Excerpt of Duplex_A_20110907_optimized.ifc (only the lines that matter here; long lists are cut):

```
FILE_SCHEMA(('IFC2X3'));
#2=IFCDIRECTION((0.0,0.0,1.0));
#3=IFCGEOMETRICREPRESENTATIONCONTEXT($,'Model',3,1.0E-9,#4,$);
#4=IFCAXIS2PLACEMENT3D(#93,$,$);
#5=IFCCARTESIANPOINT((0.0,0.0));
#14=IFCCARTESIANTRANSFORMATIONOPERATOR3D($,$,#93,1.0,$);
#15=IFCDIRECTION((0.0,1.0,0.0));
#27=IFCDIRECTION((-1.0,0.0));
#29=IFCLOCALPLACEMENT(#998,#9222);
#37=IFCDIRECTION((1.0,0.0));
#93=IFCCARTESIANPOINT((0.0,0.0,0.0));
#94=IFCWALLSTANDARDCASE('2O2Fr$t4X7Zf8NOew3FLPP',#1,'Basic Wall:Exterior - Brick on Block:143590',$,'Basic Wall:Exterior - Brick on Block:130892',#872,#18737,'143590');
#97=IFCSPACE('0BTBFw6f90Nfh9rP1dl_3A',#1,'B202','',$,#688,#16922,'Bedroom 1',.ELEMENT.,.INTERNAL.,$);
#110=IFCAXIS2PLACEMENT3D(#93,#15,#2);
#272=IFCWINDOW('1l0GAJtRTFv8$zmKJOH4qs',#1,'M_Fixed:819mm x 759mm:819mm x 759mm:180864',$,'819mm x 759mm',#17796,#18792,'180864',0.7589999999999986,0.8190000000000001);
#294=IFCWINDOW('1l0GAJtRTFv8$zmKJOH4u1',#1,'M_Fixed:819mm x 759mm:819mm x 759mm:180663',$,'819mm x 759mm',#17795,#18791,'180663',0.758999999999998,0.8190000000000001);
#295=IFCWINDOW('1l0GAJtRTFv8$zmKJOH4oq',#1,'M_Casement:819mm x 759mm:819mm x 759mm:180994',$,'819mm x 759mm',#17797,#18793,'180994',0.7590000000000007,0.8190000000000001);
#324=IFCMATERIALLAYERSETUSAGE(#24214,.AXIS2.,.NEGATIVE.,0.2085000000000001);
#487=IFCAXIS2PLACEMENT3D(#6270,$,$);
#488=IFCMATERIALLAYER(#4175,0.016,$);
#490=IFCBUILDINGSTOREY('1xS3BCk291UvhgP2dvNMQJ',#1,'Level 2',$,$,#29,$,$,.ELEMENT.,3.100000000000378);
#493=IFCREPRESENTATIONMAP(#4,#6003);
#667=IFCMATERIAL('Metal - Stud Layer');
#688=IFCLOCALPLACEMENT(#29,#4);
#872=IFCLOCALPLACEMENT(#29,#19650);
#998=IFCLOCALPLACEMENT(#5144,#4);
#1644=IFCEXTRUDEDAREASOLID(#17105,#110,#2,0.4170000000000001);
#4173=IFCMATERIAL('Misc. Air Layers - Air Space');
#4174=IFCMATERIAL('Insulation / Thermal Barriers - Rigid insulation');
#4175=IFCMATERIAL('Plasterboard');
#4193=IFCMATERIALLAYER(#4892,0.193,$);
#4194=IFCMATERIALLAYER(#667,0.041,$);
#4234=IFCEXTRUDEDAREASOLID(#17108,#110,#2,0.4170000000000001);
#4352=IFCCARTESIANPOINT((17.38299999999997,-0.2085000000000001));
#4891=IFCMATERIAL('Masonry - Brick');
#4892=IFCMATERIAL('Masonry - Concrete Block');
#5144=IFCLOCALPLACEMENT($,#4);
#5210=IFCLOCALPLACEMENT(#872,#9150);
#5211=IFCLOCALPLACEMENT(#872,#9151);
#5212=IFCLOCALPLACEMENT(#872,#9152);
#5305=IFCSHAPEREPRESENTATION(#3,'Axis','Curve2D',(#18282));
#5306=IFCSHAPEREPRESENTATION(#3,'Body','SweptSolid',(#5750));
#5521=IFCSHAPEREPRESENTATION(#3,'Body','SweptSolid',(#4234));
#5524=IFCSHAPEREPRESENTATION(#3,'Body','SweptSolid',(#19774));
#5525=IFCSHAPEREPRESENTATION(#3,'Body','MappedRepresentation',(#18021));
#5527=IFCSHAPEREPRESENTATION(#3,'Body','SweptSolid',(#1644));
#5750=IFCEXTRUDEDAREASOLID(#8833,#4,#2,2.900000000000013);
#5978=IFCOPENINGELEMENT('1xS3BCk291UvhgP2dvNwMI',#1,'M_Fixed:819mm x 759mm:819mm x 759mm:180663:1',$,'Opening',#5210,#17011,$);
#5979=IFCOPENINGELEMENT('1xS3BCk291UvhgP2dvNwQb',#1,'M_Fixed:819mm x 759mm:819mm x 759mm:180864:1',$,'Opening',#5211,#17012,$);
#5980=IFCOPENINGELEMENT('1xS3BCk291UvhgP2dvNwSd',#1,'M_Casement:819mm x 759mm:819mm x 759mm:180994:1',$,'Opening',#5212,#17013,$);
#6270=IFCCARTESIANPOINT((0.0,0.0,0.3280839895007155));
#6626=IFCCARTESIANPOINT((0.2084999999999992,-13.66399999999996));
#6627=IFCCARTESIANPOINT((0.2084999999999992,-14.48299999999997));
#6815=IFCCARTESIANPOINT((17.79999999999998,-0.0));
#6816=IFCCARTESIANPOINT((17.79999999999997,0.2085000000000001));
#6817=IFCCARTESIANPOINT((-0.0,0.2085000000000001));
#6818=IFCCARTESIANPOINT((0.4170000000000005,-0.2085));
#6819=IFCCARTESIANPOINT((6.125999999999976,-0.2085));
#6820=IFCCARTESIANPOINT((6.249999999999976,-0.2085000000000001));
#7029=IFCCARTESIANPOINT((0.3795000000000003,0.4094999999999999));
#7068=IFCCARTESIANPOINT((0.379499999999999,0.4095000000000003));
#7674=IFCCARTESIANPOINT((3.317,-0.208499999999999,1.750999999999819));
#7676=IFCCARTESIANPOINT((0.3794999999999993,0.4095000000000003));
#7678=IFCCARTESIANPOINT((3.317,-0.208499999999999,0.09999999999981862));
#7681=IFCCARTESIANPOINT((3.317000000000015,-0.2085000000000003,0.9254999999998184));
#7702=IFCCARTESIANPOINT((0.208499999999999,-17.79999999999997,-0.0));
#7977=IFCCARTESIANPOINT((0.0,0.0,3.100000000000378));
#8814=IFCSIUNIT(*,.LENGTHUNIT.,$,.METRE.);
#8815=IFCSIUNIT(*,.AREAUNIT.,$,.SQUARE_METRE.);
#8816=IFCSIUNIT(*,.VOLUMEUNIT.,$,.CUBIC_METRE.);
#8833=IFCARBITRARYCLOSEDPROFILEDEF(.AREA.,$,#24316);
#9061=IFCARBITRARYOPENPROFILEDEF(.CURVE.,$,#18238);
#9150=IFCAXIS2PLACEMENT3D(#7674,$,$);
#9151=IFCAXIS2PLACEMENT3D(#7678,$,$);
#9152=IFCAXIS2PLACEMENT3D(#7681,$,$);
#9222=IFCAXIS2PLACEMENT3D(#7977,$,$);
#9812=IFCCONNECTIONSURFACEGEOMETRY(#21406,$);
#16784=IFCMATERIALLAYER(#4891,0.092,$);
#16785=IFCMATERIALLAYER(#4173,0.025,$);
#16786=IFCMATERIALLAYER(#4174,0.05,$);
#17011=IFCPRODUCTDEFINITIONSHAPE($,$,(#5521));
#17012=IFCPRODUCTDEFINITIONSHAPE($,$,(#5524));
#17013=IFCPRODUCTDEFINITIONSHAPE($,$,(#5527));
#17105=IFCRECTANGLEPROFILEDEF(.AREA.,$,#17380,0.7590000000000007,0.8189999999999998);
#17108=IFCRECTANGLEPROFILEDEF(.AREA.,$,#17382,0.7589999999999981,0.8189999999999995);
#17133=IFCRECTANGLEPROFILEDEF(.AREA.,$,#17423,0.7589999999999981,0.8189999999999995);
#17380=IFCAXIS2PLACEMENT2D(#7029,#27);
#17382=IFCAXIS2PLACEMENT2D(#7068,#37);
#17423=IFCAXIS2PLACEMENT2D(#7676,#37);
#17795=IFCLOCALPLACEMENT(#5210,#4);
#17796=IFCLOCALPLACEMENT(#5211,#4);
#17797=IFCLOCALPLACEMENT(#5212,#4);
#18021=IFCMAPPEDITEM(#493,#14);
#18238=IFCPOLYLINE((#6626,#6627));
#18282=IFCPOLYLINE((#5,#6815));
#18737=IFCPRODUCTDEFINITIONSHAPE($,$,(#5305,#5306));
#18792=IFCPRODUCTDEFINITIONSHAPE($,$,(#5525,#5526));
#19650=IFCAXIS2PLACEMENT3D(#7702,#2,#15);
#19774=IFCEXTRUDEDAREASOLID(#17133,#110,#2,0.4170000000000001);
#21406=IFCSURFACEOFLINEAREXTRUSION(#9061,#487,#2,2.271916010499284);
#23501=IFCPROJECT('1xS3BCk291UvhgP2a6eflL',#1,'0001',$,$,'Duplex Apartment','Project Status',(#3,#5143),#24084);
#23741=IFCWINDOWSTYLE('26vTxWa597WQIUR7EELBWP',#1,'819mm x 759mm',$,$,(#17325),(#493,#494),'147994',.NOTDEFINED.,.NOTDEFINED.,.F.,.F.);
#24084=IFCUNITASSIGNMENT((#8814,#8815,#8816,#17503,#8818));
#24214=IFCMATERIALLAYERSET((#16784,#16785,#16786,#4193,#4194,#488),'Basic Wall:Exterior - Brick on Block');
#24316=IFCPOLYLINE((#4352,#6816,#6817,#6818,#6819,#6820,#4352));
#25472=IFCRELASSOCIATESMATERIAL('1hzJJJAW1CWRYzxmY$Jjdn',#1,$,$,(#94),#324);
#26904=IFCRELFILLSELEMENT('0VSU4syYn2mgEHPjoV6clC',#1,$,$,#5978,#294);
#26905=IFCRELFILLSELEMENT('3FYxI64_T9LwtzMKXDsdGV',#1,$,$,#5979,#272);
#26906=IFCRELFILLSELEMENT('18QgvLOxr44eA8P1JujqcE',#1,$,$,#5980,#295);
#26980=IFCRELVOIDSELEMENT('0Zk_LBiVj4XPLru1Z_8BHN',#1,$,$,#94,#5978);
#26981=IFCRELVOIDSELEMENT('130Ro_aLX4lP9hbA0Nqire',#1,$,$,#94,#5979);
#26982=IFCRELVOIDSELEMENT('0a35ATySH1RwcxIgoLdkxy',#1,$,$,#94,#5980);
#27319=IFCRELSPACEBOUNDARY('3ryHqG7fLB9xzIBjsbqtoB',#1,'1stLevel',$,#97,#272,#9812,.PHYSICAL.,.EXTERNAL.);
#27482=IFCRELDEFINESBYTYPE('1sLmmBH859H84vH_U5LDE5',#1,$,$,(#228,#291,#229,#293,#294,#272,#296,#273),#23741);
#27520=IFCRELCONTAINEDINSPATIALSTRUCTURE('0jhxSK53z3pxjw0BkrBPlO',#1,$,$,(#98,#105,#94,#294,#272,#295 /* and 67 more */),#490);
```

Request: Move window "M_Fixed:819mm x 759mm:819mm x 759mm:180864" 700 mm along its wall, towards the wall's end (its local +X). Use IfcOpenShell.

```python
import numpy as np
import ifcopenshell
import ifcopenshell.api.geometry
import ifcopenshell.util.placement

model = ifcopenshell.open("Duplex_A_20110907_optimized.ifc")

window = model.by_guid("1l0GAJtRTFv8$zmKJOH4qs")
opening = window.FillsVoids[0].RelatingOpeningElement
wall = opening.VoidsElements[0].RelatingBuildingElement

wall_matrix = ifcopenshell.util.placement.get_local_placement(wall.ObjectPlacement)
shift = wall_matrix[:3, 0] * 0.7
before = ifcopenshell.util.placement.get_local_placement(window.ObjectPlacement)[:3, 3].copy()

# The window is placed relative to its opening, so it follows when the opening moves.
matrix = ifcopenshell.util.placement.get_local_placement(opening.ObjectPlacement)
matrix[:3, 3] += shift
ifcopenshell.api.geometry.edit_object_placement(
    model, product=opening, matrix=matrix, is_si=False, should_transform_children=True
)

# Space boundary surfaces are stored in each space's coordinates; move them too.
for rel in window.ProvidesBoundaries:
    if not rel.ConnectionGeometry:
        continue
    surface = rel.ConnectionGeometry.SurfaceOnRelatingElement
    space_matrix = ifcopenshell.util.placement.get_local_placement(rel.RelatingSpace.ObjectPlacement)
    point = np.array(surface.Position.Location.Coordinates) + space_matrix[:3, :3].T @ shift
    surface.Position = model.createIfcAxis2Placement3D(
        model.createIfcCartesianPoint(point.tolist()), surface.Position.Axis, surface.Position.RefDirection
    )

after = ifcopenshell.util.placement.get_local_placement(window.ObjectPlacement)[:3, 3]
print("window moved by", (after - before).round(3) + 0.0)

model.write("Duplex_A_20110907_optimized_v2.ifc")
```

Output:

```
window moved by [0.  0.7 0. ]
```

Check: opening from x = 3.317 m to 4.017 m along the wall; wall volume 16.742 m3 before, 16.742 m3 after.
